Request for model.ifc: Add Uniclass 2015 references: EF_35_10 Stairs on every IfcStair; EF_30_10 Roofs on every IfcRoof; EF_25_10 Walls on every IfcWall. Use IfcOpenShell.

First a look at what the model holds.

```python
import ifcopenshell

model = ifcopenshell.open("model.ifc")
print(model.schema)
print("classifications:", [c.Name for c in model.by_type("IfcClassification")])
for ifc_class in ("IfcDoor", "IfcRoof", "IfcStair", "IfcWall", "IfcWindow"):
    print(ifc_class, len(model.by_type(ifc_class)))
```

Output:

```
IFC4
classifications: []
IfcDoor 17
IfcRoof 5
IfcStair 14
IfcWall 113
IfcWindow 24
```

```python
import ifcopenshell
import ifcopenshell.api.classification

model = ifcopenshell.open("model.ifc")

system = ifcopenshell.api.classification.add_classification(model, classification="Uniclass 2015")

codes = {
    "IfcStair": ("EF_35_10", "Stairs"),
    "IfcRoof": ("EF_30_10", "Roofs"),
    "IfcWall": ("EF_25_10", "Walls"),
}
for ifc_class, (code, name) in codes.items():
    products = model.by_type(ifc_class)
    ifcopenshell.api.classification.add_reference(
        model, products=products, classification=system, identification=code, name=name
    )
    print(code, len(products))

model.write("model_v2.ifc")
```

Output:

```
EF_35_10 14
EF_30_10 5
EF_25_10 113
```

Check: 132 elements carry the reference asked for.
